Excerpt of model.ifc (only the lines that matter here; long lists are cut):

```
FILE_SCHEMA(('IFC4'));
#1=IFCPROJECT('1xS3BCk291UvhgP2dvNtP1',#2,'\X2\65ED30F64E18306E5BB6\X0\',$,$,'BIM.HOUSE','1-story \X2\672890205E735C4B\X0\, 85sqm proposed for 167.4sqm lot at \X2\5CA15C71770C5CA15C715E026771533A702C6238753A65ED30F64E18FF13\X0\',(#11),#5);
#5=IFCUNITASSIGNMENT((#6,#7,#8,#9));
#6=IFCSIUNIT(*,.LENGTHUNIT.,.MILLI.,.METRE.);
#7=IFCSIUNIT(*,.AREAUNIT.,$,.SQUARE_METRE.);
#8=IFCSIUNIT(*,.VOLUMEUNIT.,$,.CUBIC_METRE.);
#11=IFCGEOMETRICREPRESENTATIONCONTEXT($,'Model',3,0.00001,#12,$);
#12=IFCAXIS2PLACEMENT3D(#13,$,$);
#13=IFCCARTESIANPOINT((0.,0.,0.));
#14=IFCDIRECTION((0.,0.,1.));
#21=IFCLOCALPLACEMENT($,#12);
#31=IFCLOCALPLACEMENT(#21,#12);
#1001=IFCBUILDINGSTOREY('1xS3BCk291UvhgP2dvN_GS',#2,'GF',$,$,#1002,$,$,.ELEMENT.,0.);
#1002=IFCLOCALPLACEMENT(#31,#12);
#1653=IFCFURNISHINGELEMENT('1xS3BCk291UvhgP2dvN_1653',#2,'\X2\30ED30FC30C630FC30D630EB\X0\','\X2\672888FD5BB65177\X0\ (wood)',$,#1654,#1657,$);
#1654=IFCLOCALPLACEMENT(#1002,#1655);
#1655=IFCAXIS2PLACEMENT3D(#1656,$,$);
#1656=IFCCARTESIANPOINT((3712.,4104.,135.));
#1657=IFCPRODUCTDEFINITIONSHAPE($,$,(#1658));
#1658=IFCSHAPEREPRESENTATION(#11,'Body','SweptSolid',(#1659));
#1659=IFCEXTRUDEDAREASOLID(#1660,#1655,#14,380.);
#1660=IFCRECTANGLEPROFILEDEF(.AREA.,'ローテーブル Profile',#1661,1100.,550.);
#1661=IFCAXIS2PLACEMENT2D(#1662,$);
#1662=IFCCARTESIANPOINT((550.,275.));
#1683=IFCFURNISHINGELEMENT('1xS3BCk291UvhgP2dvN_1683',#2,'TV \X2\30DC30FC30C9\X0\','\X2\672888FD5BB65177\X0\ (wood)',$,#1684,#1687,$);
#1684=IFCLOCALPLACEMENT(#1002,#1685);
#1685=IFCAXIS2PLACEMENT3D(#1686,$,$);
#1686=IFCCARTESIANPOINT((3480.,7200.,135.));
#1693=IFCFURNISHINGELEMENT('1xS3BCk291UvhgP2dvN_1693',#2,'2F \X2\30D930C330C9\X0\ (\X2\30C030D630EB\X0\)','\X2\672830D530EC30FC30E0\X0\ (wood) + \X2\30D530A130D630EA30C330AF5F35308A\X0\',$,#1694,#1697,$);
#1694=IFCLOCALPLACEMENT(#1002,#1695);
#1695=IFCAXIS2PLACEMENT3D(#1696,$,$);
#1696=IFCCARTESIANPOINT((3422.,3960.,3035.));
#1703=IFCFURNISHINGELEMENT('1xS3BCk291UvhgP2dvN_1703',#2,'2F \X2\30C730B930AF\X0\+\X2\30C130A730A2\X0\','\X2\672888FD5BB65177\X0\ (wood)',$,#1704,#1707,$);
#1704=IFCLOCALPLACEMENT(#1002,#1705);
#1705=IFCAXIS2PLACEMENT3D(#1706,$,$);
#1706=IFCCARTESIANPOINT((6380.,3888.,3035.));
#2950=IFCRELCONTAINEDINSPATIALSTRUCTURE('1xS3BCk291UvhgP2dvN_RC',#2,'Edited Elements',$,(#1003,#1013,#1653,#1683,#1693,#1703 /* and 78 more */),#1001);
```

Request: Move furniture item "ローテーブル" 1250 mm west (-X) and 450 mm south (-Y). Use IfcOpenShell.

```python
import ifcopenshell
import ifcopenshell.api.geometry
import ifcopenshell.util.placement

model = ifcopenshell.open("model.ifc")

item = model.by_id(1653)
matrix = ifcopenshell.util.placement.get_local_placement(item.ObjectPlacement)
matrix[0, 3] -= 1250.0
matrix[1, 3] -= 450.0
ifcopenshell.api.geometry.edit_object_placement(model, product=item, matrix=matrix, is_si=False)

print(ifcopenshell.util.placement.get_local_placement(item.ObjectPlacement).round(3) + 0.0)

model.write("model-out.ifc")
```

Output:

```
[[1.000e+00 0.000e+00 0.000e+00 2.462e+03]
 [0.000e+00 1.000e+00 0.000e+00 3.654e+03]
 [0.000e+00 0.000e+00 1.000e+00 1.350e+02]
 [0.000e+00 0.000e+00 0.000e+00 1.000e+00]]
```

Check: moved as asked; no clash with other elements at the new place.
